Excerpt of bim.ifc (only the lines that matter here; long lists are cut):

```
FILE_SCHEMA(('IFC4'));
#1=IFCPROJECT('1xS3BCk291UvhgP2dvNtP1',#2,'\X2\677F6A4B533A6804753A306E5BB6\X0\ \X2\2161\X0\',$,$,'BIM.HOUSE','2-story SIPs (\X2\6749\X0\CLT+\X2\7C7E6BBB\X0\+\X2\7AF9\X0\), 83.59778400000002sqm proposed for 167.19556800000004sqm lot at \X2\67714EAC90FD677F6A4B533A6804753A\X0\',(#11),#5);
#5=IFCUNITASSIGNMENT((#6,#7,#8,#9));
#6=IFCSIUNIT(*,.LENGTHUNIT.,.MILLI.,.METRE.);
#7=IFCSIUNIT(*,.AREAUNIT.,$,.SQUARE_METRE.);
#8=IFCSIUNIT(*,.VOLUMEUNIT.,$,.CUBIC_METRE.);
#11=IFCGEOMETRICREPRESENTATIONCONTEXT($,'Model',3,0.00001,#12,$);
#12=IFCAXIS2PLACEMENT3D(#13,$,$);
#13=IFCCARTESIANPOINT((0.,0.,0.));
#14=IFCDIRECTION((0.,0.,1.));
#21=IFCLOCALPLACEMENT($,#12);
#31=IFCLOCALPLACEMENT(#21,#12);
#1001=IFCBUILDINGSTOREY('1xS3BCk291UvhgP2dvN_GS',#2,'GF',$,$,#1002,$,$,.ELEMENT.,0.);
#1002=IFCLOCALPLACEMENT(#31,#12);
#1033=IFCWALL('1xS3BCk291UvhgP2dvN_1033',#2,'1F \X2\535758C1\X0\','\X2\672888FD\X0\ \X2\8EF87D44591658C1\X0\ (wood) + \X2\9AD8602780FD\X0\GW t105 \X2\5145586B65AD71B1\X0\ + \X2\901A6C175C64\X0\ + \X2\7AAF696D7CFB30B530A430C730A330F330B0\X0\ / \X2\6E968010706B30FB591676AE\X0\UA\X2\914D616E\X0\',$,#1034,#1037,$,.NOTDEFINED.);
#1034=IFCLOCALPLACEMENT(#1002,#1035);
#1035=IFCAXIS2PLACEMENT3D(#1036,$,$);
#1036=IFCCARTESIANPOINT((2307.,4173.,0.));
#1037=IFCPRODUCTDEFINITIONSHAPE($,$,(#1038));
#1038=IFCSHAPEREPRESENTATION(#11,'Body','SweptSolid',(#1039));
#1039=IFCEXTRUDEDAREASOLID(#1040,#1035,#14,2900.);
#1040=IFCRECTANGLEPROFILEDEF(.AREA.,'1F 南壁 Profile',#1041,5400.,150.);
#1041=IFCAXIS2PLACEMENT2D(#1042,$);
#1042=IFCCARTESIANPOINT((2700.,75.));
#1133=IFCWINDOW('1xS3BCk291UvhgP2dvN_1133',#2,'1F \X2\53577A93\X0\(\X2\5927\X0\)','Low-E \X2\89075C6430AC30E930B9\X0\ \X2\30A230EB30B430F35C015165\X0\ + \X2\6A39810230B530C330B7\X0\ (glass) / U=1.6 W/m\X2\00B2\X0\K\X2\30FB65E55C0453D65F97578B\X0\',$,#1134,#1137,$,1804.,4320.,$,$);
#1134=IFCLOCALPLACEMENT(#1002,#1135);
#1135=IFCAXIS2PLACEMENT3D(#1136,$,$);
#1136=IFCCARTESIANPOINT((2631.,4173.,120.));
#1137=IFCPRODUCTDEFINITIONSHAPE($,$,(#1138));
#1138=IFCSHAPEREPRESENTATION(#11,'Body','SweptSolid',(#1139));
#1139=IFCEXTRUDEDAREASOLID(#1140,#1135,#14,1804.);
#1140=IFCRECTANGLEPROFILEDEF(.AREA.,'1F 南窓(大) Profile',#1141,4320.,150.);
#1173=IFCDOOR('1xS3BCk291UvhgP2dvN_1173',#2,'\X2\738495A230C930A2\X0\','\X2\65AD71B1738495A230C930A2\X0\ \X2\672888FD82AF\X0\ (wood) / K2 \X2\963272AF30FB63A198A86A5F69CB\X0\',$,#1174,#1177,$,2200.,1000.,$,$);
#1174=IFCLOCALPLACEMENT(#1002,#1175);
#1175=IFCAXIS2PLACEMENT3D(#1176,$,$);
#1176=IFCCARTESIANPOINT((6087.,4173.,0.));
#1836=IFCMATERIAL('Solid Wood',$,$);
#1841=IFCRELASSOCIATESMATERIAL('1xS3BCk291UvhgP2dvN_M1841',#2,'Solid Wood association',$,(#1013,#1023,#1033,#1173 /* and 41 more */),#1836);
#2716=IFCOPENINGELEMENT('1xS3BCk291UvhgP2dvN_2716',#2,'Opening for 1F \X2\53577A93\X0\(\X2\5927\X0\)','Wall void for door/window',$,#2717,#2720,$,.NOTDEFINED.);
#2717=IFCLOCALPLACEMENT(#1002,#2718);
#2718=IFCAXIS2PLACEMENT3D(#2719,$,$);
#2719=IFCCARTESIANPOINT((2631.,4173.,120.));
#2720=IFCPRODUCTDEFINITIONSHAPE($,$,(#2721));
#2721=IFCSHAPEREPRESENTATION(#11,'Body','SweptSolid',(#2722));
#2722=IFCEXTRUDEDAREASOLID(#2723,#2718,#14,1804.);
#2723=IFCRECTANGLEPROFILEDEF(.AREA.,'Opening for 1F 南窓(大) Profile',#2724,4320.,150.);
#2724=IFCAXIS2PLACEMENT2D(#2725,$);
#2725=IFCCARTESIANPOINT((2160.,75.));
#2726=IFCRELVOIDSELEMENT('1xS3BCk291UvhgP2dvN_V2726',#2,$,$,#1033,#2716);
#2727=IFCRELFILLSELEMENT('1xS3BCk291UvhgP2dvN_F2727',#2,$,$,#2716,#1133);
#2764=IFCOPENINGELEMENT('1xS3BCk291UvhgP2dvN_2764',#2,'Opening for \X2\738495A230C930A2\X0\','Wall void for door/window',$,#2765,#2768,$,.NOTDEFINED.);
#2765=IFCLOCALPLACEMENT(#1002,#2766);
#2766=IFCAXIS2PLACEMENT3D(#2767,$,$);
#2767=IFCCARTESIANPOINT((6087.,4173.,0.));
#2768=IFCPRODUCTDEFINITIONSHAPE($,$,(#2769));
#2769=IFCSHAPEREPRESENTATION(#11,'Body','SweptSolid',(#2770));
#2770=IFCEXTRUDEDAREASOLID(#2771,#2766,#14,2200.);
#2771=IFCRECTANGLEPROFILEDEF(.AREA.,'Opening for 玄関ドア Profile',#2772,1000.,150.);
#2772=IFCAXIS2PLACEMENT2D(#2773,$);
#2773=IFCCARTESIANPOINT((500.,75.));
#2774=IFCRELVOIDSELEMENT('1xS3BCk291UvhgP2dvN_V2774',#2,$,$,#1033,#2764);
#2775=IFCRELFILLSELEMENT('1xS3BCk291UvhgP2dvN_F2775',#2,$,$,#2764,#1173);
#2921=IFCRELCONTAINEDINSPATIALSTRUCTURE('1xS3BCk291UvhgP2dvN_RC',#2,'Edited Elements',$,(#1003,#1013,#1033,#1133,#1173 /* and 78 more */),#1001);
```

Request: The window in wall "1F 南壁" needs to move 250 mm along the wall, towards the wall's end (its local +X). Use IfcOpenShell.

```python
import ifcopenshell
import ifcopenshell.api.geometry
import ifcopenshell.util.placement
import ifcopenshell.util.unit

model = ifcopenshell.open("bim.ifc")
unit_scale = ifcopenshell.util.unit.calculate_unit_scale(model)

window = model.by_id(1133)
opening = window.FillsVoids[0].RelatingOpeningElement
wall = opening.VoidsElements[0].RelatingBuildingElement

wall_matrix = ifcopenshell.util.placement.get_local_placement(wall.ObjectPlacement)
shift = wall_matrix[:3, 0] * 0.25 / unit_scale
before = ifcopenshell.util.placement.get_local_placement(window.ObjectPlacement)[:3, 3].copy()

# The window is not placed relative to its opening, so move both.
for product in (opening, window):
    matrix = ifcopenshell.util.placement.get_local_placement(product.ObjectPlacement)
    matrix[:3, 3] += shift
    ifcopenshell.api.geometry.edit_object_placement(model, product=product, matrix=matrix, is_si=False)

after = ifcopenshell.util.placement.get_local_placement(window.ObjectPlacement)[:3, 3]
print("window moved by", (after - before).round(3) + 0.0)

model.write("bim-out.ifc")
```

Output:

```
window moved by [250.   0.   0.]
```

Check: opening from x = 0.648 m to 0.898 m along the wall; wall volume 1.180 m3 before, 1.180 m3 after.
